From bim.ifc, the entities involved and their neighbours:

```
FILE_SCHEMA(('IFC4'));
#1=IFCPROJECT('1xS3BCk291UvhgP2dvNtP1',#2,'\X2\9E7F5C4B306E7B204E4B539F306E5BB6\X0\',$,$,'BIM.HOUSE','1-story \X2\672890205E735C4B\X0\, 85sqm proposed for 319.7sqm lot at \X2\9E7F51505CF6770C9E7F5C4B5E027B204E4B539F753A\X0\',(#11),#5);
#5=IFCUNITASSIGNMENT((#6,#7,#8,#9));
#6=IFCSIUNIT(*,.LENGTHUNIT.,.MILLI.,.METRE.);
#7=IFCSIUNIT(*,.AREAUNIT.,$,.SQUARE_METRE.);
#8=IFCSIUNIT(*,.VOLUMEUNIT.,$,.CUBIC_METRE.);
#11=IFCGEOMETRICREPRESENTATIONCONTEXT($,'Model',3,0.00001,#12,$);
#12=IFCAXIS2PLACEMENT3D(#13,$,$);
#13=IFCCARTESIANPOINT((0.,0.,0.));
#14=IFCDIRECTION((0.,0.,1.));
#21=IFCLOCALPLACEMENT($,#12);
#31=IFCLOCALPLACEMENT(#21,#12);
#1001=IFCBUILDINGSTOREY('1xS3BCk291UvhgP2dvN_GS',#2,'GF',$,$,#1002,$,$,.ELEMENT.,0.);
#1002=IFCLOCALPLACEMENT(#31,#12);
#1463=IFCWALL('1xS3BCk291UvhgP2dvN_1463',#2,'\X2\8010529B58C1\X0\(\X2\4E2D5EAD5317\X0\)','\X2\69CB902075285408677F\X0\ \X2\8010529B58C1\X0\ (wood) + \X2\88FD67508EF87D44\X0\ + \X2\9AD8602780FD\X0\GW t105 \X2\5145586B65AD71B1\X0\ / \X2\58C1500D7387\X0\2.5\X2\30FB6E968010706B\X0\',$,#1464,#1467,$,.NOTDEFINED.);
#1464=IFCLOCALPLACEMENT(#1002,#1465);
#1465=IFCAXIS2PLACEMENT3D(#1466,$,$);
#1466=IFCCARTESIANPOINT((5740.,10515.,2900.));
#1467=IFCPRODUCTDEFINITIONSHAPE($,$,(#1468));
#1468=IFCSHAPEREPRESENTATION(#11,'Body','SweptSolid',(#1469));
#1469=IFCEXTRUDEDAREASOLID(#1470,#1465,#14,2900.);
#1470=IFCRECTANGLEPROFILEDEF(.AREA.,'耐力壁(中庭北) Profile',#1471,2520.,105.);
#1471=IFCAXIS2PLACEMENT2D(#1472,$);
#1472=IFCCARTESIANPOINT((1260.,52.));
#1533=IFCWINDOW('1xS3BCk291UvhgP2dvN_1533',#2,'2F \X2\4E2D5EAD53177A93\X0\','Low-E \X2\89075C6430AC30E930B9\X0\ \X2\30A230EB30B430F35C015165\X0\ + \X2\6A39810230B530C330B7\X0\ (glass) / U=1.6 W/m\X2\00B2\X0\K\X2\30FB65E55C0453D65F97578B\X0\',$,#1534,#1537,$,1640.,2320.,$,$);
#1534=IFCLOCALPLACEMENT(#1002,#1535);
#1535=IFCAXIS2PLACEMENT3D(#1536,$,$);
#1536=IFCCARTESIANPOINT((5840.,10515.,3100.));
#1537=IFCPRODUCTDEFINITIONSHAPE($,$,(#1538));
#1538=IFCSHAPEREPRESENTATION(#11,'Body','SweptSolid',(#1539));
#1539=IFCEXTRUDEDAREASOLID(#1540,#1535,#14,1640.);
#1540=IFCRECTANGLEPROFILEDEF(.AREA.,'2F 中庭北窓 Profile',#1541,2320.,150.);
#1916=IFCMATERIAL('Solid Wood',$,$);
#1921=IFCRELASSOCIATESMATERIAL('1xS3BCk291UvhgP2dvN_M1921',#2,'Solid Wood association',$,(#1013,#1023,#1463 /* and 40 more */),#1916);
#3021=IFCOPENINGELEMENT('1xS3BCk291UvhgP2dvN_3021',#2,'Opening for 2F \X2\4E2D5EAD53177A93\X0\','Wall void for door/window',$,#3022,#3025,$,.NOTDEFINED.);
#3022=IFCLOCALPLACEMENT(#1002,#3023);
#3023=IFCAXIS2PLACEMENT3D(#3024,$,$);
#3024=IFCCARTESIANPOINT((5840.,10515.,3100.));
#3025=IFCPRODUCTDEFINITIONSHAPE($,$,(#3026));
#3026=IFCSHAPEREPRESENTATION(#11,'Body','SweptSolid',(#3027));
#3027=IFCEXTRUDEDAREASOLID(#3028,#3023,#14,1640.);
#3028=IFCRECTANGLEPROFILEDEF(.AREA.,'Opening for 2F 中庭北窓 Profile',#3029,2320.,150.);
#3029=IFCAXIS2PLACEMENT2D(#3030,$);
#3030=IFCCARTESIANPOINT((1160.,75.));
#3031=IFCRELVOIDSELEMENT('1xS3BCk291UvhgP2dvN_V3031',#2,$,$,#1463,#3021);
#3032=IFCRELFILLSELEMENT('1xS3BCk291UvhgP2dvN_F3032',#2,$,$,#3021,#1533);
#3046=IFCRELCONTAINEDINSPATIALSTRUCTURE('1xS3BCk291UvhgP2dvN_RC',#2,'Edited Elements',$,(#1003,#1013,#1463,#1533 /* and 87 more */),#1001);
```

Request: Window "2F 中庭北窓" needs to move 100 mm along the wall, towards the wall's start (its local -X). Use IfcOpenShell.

```python
import ifcopenshell
import ifcopenshell.api.geometry
import ifcopenshell.util.placement

model = ifcopenshell.open("bim.ifc")

window = model.by_id(1533)
opening = window.FillsVoids[0].RelatingOpeningElement
wall = opening.VoidsElements[0].RelatingBuildingElement

wall_matrix = ifcopenshell.util.placement.get_local_placement(wall.ObjectPlacement)
shift = wall_matrix[:3, 0] * -100.0
before = ifcopenshell.util.placement.get_local_placement(window.ObjectPlacement)[:3, 3].copy()

# The window is not placed relative to its opening, so move both.
for product in (opening, window):
    matrix = ifcopenshell.util.placement.get_local_placement(product.ObjectPlacement)
    matrix[:3, 3] += shift
    ifcopenshell.api.geometry.edit_object_placement(model, product=product, matrix=matrix, is_si=False)

after = ifcopenshell.util.placement.get_local_placement(window.ObjectPlacement)[:3, 3]
print("window moved by", (after - before).round(3) + 0.0)

model.write("bim_updated.ifc")
```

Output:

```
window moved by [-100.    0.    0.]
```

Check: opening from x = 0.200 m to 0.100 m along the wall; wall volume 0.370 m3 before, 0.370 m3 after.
